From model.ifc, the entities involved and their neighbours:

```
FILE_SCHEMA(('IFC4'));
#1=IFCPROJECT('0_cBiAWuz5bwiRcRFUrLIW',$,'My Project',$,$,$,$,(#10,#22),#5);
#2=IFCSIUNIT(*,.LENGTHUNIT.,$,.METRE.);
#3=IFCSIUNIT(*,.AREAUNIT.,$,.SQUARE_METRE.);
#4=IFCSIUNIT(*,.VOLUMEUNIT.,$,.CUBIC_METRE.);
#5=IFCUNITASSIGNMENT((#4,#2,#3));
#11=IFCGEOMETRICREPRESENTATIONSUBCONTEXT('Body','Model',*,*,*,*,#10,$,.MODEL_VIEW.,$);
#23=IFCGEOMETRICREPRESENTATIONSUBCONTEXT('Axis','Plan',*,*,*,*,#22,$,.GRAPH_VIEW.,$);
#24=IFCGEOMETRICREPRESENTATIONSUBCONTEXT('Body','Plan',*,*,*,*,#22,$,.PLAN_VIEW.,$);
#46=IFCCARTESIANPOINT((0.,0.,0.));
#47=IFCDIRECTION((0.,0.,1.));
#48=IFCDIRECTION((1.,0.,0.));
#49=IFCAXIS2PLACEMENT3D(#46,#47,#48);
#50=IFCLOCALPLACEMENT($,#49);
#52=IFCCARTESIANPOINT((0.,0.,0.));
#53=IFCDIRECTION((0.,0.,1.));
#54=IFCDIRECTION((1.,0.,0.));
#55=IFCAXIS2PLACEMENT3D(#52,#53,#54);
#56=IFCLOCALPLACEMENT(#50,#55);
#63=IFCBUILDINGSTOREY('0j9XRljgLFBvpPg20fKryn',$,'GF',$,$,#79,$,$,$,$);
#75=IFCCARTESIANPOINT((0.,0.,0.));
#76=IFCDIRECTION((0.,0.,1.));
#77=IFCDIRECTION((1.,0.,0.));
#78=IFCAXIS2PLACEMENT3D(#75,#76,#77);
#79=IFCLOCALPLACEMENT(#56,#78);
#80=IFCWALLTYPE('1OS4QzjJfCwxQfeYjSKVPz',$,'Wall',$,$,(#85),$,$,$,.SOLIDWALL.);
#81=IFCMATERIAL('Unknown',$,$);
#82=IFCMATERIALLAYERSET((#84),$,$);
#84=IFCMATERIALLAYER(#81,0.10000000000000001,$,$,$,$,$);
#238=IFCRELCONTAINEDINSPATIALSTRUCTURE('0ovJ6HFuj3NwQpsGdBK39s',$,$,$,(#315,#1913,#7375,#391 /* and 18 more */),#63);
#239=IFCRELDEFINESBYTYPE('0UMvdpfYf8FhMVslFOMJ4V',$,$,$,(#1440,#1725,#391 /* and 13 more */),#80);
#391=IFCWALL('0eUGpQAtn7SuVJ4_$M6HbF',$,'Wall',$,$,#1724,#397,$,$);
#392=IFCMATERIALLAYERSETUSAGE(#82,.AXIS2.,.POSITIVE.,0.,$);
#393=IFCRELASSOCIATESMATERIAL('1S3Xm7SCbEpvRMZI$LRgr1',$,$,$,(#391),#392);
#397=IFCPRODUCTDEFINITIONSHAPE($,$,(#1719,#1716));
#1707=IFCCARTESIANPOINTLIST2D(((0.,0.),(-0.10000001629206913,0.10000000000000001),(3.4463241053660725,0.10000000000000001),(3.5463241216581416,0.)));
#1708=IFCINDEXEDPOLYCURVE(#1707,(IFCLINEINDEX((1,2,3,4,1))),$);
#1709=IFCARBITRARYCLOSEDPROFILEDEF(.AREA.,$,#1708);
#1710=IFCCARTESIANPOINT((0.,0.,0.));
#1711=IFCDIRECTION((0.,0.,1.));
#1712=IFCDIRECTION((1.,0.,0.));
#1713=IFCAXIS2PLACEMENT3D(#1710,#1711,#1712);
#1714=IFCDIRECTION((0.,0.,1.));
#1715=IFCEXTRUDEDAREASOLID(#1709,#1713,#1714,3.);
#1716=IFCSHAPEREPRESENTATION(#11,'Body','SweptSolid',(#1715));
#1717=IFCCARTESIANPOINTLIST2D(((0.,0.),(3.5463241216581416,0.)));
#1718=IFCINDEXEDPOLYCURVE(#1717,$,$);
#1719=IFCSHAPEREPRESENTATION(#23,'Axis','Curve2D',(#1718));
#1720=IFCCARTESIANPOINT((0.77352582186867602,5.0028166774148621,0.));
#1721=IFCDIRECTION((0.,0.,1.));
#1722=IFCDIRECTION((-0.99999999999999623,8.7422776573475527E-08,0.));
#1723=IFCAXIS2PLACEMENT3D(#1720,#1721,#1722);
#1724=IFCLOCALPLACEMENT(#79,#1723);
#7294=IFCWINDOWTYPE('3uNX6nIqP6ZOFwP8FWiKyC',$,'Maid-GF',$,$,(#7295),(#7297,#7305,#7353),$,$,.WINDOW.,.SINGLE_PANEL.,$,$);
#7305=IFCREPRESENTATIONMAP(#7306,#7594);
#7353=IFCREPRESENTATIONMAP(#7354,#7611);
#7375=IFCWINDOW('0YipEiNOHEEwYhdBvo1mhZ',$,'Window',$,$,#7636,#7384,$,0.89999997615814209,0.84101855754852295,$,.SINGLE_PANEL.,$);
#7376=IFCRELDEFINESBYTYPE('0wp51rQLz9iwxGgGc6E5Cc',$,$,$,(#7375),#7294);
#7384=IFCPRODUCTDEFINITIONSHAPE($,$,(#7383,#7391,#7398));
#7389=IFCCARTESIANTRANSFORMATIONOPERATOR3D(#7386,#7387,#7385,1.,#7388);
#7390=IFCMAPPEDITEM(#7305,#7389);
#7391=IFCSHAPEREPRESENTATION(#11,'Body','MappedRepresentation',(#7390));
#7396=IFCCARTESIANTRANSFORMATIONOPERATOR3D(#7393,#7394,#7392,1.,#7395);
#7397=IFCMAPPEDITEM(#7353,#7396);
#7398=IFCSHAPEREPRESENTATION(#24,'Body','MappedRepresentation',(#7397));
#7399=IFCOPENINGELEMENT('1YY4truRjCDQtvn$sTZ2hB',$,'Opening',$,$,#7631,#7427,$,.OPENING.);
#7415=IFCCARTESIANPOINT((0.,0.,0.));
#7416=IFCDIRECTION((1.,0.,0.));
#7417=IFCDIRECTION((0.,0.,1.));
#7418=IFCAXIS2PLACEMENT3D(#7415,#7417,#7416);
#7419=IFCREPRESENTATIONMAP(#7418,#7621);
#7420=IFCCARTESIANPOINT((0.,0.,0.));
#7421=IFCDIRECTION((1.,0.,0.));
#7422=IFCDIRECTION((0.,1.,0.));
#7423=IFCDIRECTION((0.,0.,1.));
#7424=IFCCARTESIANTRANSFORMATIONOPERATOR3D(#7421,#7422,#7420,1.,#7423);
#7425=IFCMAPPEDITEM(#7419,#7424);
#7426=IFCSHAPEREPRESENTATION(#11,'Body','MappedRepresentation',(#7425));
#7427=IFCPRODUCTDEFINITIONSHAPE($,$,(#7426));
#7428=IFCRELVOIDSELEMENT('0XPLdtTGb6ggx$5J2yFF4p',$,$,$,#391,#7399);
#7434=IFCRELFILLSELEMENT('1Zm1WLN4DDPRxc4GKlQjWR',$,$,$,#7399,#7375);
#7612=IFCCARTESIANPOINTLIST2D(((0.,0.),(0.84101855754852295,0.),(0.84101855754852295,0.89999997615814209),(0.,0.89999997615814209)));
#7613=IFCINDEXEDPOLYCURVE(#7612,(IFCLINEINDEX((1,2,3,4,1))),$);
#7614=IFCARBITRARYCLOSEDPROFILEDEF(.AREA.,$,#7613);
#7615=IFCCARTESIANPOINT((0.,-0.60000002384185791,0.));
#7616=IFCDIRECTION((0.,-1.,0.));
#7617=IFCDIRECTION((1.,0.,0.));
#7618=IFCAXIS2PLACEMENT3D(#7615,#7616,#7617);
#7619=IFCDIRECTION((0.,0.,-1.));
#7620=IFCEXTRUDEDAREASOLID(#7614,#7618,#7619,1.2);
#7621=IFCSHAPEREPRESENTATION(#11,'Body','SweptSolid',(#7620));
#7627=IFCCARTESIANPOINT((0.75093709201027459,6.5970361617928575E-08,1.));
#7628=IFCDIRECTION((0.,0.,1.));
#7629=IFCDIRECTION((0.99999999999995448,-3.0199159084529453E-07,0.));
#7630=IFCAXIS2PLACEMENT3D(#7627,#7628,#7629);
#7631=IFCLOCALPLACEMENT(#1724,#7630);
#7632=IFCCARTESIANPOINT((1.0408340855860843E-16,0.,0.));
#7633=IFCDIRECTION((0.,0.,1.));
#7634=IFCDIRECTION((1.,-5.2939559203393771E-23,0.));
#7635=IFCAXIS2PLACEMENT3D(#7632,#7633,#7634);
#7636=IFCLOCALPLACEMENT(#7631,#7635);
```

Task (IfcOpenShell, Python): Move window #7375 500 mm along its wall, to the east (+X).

```python
import ifcopenshell
import ifcopenshell.api.geometry
import ifcopenshell.util.placement
import ifcopenshell.util.unit

model = ifcopenshell.open("model.ifc")
unit_scale = ifcopenshell.util.unit.calculate_unit_scale(model)

window = model.by_guid("0YipEiNOHEEwYhdBvo1mhZ")
opening = window.FillsVoids[0].RelatingOpeningElement
wall = opening.VoidsElements[0].RelatingBuildingElement

wall_matrix = ifcopenshell.util.placement.get_local_placement(wall.ObjectPlacement)
shift = wall_matrix[:3, 0] * -0.5 / unit_scale
before = ifcopenshell.util.placement.get_local_placement(window.ObjectPlacement)[:3, 3].copy()

# The window is placed relative to its opening, so it follows when the opening moves.
matrix = ifcopenshell.util.placement.get_local_placement(opening.ObjectPlacement)
matrix[:3, 3] += shift
ifcopenshell.api.geometry.edit_object_placement(
    model, product=opening, matrix=matrix, is_si=False, should_transform_children=True
)

after = ifcopenshell.util.placement.get_local_placement(window.ObjectPlacement)[:3, 3]
print("window moved by", (after - before).round(3) + 0.0)

model.write("model_updated.ifc")
```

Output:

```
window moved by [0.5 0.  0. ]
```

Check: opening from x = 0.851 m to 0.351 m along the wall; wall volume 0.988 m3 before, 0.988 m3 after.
